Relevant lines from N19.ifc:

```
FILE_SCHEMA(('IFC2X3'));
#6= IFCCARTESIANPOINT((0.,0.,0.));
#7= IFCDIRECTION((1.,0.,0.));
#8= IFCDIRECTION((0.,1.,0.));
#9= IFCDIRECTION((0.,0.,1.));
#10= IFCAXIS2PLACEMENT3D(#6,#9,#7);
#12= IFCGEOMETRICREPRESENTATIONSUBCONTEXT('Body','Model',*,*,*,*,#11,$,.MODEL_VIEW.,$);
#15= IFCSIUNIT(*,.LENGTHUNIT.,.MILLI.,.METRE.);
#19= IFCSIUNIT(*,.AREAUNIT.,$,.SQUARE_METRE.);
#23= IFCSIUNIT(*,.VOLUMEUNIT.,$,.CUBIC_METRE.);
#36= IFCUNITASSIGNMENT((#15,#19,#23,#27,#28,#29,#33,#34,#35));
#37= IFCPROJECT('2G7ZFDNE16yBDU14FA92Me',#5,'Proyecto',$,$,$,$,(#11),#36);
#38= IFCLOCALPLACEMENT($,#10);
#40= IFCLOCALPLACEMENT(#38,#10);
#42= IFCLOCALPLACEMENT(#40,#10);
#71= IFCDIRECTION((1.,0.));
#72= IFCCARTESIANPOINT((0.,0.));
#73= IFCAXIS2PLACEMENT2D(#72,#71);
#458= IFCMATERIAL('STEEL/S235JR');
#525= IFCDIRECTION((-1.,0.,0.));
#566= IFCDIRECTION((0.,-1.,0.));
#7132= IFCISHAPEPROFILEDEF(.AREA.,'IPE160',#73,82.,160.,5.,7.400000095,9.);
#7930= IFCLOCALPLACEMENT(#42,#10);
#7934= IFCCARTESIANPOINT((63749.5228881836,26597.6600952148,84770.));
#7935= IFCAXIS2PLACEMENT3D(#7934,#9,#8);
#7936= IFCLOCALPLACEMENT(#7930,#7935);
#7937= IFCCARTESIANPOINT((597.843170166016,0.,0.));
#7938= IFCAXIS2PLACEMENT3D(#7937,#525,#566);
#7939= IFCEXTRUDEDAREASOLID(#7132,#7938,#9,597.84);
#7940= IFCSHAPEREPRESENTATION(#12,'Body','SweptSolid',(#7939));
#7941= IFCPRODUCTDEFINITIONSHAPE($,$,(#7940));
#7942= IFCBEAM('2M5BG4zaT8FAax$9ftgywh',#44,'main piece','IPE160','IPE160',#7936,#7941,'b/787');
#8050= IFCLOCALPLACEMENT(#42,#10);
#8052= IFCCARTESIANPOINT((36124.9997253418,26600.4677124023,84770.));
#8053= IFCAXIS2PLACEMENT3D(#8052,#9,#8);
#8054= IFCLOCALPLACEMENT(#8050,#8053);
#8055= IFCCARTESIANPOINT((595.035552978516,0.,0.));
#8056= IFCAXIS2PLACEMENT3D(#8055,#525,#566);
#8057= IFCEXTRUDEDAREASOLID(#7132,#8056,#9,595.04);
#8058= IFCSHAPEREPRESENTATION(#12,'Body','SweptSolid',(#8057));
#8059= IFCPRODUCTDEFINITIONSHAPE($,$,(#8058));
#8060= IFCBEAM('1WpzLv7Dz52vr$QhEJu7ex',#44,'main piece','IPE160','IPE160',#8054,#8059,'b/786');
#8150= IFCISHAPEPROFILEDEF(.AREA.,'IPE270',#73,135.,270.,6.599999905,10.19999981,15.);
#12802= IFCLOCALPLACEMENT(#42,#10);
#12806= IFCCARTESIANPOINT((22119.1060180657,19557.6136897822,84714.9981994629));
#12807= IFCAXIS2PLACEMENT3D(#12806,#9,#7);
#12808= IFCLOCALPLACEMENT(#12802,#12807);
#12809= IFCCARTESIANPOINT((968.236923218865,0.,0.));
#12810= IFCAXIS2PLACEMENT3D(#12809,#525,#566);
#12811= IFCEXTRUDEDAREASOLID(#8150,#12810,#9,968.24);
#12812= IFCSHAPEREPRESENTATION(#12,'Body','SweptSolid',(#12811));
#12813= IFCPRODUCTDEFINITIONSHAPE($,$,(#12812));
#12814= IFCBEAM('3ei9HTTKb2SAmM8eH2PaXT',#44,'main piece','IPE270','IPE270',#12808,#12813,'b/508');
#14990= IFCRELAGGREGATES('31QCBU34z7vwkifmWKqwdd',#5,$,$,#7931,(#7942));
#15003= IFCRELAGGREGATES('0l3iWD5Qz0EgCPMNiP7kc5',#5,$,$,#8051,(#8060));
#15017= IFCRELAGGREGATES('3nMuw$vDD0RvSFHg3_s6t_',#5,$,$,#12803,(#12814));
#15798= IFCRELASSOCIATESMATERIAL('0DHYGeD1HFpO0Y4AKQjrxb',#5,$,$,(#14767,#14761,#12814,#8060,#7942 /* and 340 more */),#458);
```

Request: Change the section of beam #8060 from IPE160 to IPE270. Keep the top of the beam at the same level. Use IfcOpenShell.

```python
import ifcopenshell
import ifcopenshell.util.element
import ifcopenshell.util.representation

model = ifcopenshell.open("N19.ifc")

member = model.by_guid("1WpzLv7Dz52vr$QhEJu7ex")
source = next(p for p in model.by_type("IfcIShapeProfileDef") if p.ProfileName == "IPE270")

body = ifcopenshell.util.representation.get_representation(member, "Model", "Body")
solid = body.Items[0]
old_profile = solid.SweptArea

# Copy the section's sizes but keep this member's own profile position.
profile = ifcopenshell.util.element.copy(model, source)
# Profiles are centred, so shift by half the change in depth to hold the top.
shift = (old_profile.OverallDepth - profile.OverallDepth) / 2
x, y = old_profile.Position.Location.Coordinates
up = (0.0, 1.0)  # upwards, in the solid's own plane
location = model.createIfcCartesianPoint((x + up[0] * shift, y + up[1] * shift))
profile.Position = model.createIfcAxis2Placement2D(location, old_profile.Position.RefDirection)
solid.SweptArea = profile
if not model.get_total_inverses(old_profile):
    ifcopenshell.util.element.remove_deep2(model, old_profile)
member.Description = member.Description.replace("IPE160", "IPE270")
member.ObjectType = member.ObjectType.replace("IPE160", "IPE270")

print(solid.SweptArea)

model.write("N19_rev.ifc")
```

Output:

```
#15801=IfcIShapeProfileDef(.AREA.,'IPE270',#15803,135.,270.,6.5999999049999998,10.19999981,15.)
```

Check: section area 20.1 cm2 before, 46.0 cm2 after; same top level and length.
